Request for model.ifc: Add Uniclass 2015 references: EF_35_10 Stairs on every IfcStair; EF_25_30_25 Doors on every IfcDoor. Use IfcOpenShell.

First a look at what the model holds.

```python
import ifcopenshell

model = ifcopenshell.open("model.ifc")
print(model.schema)
print("classifications:", [c.Name for c in model.by_type("IfcClassification")])
for ifc_class in ("IfcDoor", "IfcRoof", "IfcStair", "IfcWall", "IfcWindow"):
    print(ifc_class, len(model.by_type(ifc_class)))
```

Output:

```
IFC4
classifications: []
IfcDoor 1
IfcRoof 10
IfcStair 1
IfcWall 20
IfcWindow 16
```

```python
import ifcopenshell
import ifcopenshell.api.classification

model = ifcopenshell.open("model.ifc")

system = ifcopenshell.api.classification.add_classification(model, classification="Uniclass 2015")

codes = {
    "IfcStair": ("EF_35_10", "Stairs"),
    "IfcDoor": ("EF_25_30_25", "Doors"),
}
for ifc_class, (code, name) in codes.items():
    products = model.by_type(ifc_class)
    ifcopenshell.api.classification.add_reference(
        model, products=products, classification=system, identification=code, name=name
    )
    print(code, len(products))

model.write("model-out.ifc")
```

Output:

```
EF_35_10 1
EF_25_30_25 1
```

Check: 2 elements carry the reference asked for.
